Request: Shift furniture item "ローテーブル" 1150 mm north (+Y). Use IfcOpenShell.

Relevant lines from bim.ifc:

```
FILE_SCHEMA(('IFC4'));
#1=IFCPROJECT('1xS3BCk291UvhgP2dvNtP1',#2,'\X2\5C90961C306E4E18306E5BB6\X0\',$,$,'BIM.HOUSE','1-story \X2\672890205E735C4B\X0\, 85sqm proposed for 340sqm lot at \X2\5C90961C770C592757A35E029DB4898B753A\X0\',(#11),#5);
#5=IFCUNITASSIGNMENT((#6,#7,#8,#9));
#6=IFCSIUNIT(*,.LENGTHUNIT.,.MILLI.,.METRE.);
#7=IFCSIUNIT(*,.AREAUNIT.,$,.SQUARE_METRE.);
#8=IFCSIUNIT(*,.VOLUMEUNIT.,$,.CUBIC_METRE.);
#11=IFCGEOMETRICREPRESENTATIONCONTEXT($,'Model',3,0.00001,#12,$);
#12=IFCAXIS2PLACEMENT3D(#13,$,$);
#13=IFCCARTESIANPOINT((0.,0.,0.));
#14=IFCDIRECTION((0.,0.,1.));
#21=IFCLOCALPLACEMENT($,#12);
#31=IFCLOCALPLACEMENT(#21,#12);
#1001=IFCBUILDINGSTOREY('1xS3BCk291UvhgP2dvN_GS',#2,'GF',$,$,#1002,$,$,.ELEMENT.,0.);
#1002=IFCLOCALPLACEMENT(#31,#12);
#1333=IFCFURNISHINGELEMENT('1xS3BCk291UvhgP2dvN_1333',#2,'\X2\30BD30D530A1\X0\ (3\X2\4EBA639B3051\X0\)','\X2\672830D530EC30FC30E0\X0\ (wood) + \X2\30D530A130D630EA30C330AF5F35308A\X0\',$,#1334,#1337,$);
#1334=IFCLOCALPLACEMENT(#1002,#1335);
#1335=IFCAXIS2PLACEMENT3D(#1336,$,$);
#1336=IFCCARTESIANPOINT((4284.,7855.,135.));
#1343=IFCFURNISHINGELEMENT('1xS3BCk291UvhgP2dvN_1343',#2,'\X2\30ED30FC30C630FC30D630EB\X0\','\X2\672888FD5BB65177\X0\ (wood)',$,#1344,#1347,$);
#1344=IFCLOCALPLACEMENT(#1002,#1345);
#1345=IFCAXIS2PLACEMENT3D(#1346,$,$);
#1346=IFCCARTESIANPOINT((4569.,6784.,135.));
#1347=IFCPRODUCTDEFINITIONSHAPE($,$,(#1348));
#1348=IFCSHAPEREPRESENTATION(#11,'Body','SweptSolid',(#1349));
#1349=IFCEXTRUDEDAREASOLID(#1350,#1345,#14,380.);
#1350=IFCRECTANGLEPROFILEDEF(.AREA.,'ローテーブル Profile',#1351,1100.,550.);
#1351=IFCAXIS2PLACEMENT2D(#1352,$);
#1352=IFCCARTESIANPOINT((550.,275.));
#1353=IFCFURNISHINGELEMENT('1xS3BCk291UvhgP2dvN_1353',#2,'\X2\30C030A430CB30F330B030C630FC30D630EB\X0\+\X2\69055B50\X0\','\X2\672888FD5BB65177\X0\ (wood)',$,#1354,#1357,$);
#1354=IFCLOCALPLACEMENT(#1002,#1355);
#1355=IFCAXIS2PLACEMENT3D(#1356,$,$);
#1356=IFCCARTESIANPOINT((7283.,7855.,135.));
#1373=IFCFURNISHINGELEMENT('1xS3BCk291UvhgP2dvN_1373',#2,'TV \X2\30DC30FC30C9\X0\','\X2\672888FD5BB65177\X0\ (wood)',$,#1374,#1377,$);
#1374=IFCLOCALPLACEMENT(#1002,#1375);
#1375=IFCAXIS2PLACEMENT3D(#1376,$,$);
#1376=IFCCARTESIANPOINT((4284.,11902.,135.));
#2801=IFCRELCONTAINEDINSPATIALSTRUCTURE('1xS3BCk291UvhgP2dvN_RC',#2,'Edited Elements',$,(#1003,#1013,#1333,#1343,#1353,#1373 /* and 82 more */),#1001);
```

```python
import ifcopenshell
import ifcopenshell.api.geometry
import ifcopenshell.util.placement
import ifcopenshell.util.unit

model = ifcopenshell.open("bim.ifc")
unit_scale = ifcopenshell.util.unit.calculate_unit_scale(model)

item = model.by_guid("1xS3BCk291UvhgP2dvN_1343")
matrix = ifcopenshell.util.placement.get_local_placement(item.ObjectPlacement)
matrix[1, 3] += 1.15 / unit_scale
ifcopenshell.api.geometry.edit_object_placement(model, product=item, matrix=matrix, is_si=False)

print(ifcopenshell.util.placement.get_local_placement(item.ObjectPlacement).round(3) + 0.0)

model.write("bim_v2.ifc")
```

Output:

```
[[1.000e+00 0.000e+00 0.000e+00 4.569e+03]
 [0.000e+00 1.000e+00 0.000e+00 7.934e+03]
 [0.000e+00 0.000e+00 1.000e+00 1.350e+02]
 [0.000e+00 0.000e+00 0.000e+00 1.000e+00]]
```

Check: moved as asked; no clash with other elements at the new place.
